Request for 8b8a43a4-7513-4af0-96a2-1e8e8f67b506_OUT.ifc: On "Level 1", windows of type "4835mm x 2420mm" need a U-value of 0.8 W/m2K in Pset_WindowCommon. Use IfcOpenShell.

First a look at what the model holds.

```python
import ifcopenshell
import ifcopenshell.util.element

model = ifcopenshell.open("8b8a43a4-7513-4af0-96a2-1e8e8f67b506_OUT.ifc")
print(model.schema)
storey = next(s for s in model.by_type("IfcBuildingStorey") if s.Name == "Level 1")
windows = [e for e in ifcopenshell.util.element.get_decomposition(storey) if e.is_a("IfcWindow")]
seen = {}
for e in windows:
    element_type = ifcopenshell.util.element.get_type(e)
    key = (element_type.Name if element_type != e and element_type else None, ifcopenshell.util.element.get_pset(e, "Pset_WindowCommon", "ThermalTransmittance"))
    seen[key] = seen.get(key, 0) + 1
for (name, value), count in sorted(seen.items(), key=str):
    print(count, "x", name, "|", value)
```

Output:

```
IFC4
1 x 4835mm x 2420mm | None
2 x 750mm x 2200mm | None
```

```python
import ifcopenshell
import ifcopenshell.api.pset
import ifcopenshell.util.element

model = ifcopenshell.open("8b8a43a4-7513-4af0-96a2-1e8e8f67b506_OUT.ifc")

storey = next(s for s in model.by_type("IfcBuildingStorey") if s.Name == "Level 1")
windows = [e for e in ifcopenshell.util.element.get_decomposition(storey) if e.is_a("IfcWindow")]

count = 0
for e in windows:
    element_type = ifcopenshell.util.element.get_type(e)
    if element_type in (None, e) or element_type.Name != "4835mm x 2420mm":
        continue
    # add_pset returns the element's existing set when there is one.
    pset = ifcopenshell.api.pset.add_pset(model, product=e, name="Pset_WindowCommon")
    ifcopenshell.api.pset.edit_pset(model, pset=pset, properties={"ThermalTransmittance": 0.8})
    count += 1

print(count, "windows updated")

model.write("8b8a43a4-7513-4af0-96a2-1e8e8f67b506_OUT_edited.ifc")
```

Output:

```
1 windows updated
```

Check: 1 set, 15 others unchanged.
